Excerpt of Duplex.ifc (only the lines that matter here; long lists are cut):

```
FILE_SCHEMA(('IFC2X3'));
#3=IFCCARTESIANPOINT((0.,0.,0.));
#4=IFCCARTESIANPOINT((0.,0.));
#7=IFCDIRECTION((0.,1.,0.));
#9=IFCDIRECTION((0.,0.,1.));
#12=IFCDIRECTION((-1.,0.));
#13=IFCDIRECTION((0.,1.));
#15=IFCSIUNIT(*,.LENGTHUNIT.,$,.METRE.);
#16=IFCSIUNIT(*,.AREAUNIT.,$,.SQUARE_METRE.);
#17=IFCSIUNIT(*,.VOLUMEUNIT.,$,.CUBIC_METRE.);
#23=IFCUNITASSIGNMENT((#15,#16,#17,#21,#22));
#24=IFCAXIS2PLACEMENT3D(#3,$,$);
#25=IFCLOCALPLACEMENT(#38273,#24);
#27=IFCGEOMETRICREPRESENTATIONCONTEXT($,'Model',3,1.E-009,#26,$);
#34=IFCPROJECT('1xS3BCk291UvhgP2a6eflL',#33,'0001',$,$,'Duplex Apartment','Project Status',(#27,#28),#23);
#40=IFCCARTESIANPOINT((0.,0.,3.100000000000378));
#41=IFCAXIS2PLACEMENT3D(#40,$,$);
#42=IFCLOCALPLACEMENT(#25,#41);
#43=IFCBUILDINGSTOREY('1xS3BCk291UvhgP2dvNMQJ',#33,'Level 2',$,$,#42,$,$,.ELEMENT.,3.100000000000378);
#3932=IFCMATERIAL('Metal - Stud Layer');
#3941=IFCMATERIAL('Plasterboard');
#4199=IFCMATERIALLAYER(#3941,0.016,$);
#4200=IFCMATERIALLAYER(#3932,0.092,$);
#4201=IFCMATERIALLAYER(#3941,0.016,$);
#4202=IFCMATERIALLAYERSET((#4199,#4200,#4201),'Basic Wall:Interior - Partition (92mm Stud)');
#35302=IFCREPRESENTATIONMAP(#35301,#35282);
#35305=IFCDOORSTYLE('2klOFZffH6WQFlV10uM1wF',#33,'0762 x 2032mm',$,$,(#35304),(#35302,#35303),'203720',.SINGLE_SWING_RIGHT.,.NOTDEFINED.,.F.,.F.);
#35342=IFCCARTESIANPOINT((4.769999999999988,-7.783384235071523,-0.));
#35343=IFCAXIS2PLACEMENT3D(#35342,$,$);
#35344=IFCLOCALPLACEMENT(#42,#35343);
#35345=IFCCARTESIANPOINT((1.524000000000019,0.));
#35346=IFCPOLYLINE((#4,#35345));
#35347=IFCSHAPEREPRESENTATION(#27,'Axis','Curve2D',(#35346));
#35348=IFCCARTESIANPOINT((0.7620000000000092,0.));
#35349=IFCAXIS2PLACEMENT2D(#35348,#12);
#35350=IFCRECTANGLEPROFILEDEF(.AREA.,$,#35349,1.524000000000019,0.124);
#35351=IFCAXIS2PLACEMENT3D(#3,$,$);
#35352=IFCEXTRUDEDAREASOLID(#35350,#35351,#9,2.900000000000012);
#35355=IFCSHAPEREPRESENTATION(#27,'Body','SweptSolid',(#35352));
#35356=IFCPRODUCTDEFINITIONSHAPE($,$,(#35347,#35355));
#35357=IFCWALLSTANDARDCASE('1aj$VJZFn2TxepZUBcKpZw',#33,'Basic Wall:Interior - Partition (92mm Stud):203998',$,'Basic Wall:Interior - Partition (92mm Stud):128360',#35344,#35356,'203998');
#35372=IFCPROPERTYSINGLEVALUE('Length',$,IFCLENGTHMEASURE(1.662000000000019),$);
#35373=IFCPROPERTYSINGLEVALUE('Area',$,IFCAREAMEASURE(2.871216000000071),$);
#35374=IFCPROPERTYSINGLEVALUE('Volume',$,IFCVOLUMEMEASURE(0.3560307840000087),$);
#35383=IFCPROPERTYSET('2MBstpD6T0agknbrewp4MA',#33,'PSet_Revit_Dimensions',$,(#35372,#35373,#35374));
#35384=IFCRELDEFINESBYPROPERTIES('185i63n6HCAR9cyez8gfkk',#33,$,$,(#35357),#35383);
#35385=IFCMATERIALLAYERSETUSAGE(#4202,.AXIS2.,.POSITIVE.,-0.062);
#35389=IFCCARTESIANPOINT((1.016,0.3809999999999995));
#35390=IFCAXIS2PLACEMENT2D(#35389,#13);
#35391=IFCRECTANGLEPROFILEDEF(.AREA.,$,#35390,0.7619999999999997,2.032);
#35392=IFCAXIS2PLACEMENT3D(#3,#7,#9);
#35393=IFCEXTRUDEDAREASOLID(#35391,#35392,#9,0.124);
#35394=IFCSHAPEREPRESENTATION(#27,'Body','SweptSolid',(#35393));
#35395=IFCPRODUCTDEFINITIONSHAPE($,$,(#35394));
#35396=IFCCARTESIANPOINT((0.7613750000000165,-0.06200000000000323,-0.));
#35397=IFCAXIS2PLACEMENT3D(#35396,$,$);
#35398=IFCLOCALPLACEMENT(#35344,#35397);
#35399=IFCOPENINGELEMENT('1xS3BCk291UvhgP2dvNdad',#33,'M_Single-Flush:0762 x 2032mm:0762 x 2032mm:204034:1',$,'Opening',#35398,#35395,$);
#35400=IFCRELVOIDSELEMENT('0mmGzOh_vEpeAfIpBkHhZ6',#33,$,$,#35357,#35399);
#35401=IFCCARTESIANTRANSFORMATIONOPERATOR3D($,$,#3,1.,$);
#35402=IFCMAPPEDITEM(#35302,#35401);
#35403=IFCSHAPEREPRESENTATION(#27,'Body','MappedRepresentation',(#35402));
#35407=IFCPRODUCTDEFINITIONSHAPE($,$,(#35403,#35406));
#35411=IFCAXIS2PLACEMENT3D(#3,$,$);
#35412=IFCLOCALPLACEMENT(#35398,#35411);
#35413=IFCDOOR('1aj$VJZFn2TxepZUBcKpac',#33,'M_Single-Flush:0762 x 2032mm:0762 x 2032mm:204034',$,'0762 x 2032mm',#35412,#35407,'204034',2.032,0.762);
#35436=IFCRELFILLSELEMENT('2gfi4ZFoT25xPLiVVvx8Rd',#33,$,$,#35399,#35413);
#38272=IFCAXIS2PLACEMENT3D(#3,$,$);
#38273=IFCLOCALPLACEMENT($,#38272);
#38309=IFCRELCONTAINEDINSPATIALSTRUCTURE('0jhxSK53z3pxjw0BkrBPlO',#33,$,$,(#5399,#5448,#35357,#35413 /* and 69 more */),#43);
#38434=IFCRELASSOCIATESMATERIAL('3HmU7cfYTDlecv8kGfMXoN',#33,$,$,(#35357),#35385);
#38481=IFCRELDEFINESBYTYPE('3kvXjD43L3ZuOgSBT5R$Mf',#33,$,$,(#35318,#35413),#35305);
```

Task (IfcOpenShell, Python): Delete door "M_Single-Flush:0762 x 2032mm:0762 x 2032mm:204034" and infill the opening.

```python
import ifcopenshell
import ifcopenshell.api.feature
import ifcopenshell.api.pset
import ifcopenshell.api.root
import ifcopenshell.geom
import ifcopenshell.util.element
import ifcopenshell.util.shape
import ifcopenshell.util.unit

model = ifcopenshell.open("Duplex.ifc")
area_scale = ifcopenshell.util.unit.calculate_unit_scale(model, "AREAUNIT")
volume_scale = ifcopenshell.util.unit.calculate_unit_scale(model, "VOLUMEUNIT")
settings = ifcopenshell.geom.settings()


def volume(element):
    """Net volume in cubic metres, openings subtracted."""
    shape = ifcopenshell.geom.create_shape(settings, element)
    return ifcopenshell.util.shape.get_volume(shape.geometry)


door = model.by_guid("1aj$VJZFn2TxepZUBcKpac")
opening = door.FillsVoids[0].RelatingOpeningElement
wall = opening.VoidsElements[0].RelatingBuildingElement
before = volume(wall)

ifcopenshell.api.root.remove_product(model, product=door)
ifcopenshell.api.feature.remove_feature(model, feature=opening)

after = volume(wall)
thickness = 0.124  # wall thickness in metres

# Update the wall's stored quantities.
pset = model.by_id(ifcopenshell.util.element.get_pset(wall, "PSet_Revit_Dimensions", should_inherit=False)["id"])
ifcopenshell.api.pset.edit_pset(model, pset=pset, properties={
    "Area": model.create_entity("IfcAreaMeasure", after / thickness / area_scale),
    "Volume": model.create_entity("IfcVolumeMeasure", after / volume_scale),
})

print(f"wall volume {before:.3f} -> {after:.3f} m3")

model.write("Duplex_edited.ifc")
```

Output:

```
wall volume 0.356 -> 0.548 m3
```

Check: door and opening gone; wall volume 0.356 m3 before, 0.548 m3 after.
